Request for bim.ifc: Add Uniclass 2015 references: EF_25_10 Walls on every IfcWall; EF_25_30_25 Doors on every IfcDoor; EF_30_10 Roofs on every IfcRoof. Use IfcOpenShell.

First a look at what the model holds.

```python
import ifcopenshell

model = ifcopenshell.open("bim.ifc")
print(model.schema)
print("classifications:", [c.Name for c in model.by_type("IfcClassification")])
for ifc_class in ("IfcDoor", "IfcRoof", "IfcStair", "IfcWall", "IfcWindow"):
    print(ifc_class, len(model.by_type(ifc_class)))
```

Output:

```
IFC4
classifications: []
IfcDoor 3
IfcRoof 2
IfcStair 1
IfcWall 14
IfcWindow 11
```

```python
import ifcopenshell
import ifcopenshell.api.classification

model = ifcopenshell.open("bim.ifc")

system = ifcopenshell.api.classification.add_classification(model, classification="Uniclass 2015")

codes = {
    "IfcWall": ("EF_25_10", "Walls"),
    "IfcDoor": ("EF_25_30_25", "Doors"),
    "IfcRoof": ("EF_30_10", "Roofs"),
}
for ifc_class, (code, name) in codes.items():
    products = model.by_type(ifc_class)
    ifcopenshell.api.classification.add_reference(
        model, products=products, classification=system, identification=code, name=name
    )
    print(code, len(products))

model.write("bim_rev.ifc")
```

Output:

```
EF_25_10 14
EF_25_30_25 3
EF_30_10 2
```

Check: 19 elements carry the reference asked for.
